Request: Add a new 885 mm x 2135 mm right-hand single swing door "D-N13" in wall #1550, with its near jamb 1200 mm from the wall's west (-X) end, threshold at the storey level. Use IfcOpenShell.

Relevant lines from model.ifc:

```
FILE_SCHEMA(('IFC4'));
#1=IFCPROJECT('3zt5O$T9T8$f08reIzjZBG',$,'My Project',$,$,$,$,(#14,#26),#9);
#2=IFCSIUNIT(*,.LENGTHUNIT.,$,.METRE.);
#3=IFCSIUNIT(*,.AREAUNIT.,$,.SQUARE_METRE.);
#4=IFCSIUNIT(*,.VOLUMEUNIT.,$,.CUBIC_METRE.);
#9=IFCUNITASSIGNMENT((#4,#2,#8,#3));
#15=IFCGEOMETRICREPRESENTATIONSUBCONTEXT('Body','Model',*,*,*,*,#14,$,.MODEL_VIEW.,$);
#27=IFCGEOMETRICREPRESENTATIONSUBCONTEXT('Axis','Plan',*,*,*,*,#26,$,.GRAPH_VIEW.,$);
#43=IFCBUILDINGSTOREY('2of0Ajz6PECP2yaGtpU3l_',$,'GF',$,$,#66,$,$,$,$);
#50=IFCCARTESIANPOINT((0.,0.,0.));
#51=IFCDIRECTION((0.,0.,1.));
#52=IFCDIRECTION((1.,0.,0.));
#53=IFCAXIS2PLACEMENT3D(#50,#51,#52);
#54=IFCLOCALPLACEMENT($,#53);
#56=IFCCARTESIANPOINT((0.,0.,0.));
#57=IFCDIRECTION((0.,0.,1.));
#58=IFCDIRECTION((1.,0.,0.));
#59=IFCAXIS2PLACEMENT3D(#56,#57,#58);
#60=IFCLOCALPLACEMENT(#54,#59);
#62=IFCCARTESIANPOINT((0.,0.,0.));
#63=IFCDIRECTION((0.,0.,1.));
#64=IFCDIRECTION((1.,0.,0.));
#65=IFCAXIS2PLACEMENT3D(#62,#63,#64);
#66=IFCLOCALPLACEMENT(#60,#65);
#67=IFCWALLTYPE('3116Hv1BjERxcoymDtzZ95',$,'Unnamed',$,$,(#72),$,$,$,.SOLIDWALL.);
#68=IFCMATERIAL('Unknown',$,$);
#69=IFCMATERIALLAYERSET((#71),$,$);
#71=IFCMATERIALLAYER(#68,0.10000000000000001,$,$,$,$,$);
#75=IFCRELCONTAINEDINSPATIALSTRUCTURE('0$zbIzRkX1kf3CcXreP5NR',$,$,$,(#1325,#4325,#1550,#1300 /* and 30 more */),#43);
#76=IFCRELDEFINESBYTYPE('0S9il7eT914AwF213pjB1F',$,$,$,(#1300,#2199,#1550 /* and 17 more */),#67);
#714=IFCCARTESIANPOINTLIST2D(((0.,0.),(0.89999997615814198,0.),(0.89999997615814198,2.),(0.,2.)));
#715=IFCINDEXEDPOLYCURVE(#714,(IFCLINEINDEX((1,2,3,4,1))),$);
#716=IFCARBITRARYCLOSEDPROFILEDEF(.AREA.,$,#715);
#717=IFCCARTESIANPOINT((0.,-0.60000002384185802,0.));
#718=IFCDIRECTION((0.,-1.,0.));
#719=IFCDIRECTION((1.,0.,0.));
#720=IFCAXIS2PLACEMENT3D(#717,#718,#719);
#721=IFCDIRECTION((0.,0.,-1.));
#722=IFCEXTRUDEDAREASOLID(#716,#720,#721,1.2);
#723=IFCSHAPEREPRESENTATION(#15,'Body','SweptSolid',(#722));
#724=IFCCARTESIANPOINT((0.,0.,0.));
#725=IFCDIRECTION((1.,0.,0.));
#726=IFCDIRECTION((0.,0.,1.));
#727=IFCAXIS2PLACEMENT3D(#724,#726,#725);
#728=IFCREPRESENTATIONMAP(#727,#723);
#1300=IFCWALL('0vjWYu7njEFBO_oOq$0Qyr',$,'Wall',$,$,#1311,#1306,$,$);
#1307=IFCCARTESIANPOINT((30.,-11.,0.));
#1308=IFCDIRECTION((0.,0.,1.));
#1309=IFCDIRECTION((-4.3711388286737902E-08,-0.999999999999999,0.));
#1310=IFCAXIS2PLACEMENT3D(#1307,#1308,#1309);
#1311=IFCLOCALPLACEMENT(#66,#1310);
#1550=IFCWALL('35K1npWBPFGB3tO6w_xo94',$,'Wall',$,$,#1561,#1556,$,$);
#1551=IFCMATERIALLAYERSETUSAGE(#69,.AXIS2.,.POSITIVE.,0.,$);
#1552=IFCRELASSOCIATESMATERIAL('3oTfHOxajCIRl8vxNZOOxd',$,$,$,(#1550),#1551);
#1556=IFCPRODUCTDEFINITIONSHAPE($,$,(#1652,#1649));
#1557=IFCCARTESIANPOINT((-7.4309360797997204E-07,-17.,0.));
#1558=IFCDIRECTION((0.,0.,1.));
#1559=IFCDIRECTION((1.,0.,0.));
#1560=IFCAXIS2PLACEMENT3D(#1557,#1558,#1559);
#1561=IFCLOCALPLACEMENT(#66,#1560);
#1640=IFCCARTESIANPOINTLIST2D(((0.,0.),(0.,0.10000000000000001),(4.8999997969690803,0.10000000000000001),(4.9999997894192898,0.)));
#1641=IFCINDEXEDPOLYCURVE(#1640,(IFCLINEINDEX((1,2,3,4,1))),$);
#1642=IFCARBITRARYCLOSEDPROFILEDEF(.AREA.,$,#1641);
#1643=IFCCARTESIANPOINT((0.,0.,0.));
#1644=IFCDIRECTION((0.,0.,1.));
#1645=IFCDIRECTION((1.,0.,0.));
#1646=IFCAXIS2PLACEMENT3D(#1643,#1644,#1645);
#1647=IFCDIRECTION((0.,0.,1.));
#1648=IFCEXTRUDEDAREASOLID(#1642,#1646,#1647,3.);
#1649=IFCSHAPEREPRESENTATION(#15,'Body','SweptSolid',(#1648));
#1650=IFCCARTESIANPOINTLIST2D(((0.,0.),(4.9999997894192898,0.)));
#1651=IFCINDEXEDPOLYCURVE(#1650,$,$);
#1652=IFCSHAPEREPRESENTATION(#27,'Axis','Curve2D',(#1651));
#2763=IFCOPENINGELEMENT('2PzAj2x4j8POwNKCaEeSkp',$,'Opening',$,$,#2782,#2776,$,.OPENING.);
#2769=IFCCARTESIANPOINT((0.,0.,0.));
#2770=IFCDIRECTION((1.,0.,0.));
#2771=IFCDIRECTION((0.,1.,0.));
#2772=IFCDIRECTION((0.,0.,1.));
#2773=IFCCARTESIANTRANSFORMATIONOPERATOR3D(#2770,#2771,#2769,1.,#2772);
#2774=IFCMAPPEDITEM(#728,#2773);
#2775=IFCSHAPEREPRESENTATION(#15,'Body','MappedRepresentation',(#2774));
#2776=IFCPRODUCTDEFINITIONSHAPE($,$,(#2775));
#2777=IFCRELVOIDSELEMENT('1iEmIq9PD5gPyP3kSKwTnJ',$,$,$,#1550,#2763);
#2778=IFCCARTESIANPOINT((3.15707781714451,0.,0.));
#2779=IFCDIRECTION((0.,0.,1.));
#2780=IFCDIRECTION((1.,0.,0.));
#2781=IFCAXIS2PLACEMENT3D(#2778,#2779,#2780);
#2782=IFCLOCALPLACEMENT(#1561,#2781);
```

```python
import numpy as np
import ifcopenshell
import ifcopenshell.api.feature
import ifcopenshell.api.geometry
import ifcopenshell.api.root
import ifcopenshell.api.spatial
import ifcopenshell.geom
import ifcopenshell.util.element
import ifcopenshell.util.placement
import ifcopenshell.util.representation
import ifcopenshell.util.shape
import ifcopenshell.util.unit

model = ifcopenshell.open("model.ifc")
unit_scale = ifcopenshell.util.unit.calculate_unit_scale(model)
settings = ifcopenshell.geom.settings()


def volume(element):
    """Net volume in cubic metres, openings subtracted."""
    shape = ifcopenshell.geom.create_shape(settings, element)
    return ifcopenshell.util.shape.get_volume(shape.geometry)


wall = model.by_guid("35K1npWBPFGB3tO6w_xo94")
storey = ifcopenshell.util.element.get_container(wall, ifc_class="IfcBuildingStorey")
context = ifcopenshell.util.representation.get_context(model, "Model", "Body", "MODEL_VIEW")
before = volume(wall)

width, height, from_end, sill = 0.885, 2.135, 1.2, 0.0  # metres

# The wall runs along its own X axis, and the end named is its -X end.
wall_shape = ifcopenshell.geom.create_shape(settings, wall)
x, y, z = ifcopenshell.util.shape.get_vertices(wall_shape.geometry).T
start = x.min() + from_end
face, thickness = float(y.min()), float(y.max() - y.min())
wall_matrix = ifcopenshell.util.placement.get_local_placement(wall.ObjectPlacement)
level = ifcopenshell.util.placement.get_local_placement(storey.ObjectPlacement)[2, 3]


def in_wall(x, y):
    """Placement at x, y metres in the wall's axes, at sill height."""
    matrix = wall_matrix.copy()
    matrix[:, 3] = wall_matrix @ np.array([x / unit_scale, y / unit_scale, 0.0, 1.0])
    matrix[2, 3] = level + sill / unit_scale
    return matrix


# Opening: a box that overshoots both wall faces by 50 mm.
opening = ifcopenshell.api.root.create_entity(model, ifc_class="IfcOpeningElement", predefined_type="OPENING")
box = ifcopenshell.api.geometry.add_wall_representation(
    model, context=context, length=width, height=height, thickness=thickness + 0.1
)
ifcopenshell.api.geometry.assign_representation(model, product=opening, representation=box)
ifcopenshell.api.geometry.edit_object_placement(model, product=opening, matrix=in_wall(start, face - 0.05), is_si=False)
ifcopenshell.api.feature.add_feature(model, feature=opening, element=wall)

door = ifcopenshell.api.root.create_entity(model, ifc_class="IfcDoor", name="D-N13", predefined_type="DOOR")
door.OverallWidth, door.OverallHeight = width / unit_scale, height / unit_scale
door.OperationType = "SINGLE_SWING_RIGHT"
body = ifcopenshell.api.geometry.add_door_representation(
    model,
    context=context,
    overall_width=door.OverallWidth,
    overall_height=door.OverallHeight,
    operation_type="SINGLE_SWING_RIGHT",
    lining_properties={"LiningDepth": thickness / unit_scale, "ThresholdDepth": thickness / unit_scale},
)
ifcopenshell.api.geometry.assign_representation(model, product=door, representation=body)
ifcopenshell.api.spatial.assign_container(model, products=[door], relating_structure=storey)
ifcopenshell.api.feature.add_filling(model, opening=opening, element=door)

# The lining spans the wall, so the door starts at the wall face.
ifcopenshell.api.geometry.edit_object_placement(model, product=door, matrix=in_wall(start, face), is_si=False)

after = volume(wall)

print(f"wall volume {before:.3f} -> {after:.3f} m3")

model.write("model_edited.ifc")
```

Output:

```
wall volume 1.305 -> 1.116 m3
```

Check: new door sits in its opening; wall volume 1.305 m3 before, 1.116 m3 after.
